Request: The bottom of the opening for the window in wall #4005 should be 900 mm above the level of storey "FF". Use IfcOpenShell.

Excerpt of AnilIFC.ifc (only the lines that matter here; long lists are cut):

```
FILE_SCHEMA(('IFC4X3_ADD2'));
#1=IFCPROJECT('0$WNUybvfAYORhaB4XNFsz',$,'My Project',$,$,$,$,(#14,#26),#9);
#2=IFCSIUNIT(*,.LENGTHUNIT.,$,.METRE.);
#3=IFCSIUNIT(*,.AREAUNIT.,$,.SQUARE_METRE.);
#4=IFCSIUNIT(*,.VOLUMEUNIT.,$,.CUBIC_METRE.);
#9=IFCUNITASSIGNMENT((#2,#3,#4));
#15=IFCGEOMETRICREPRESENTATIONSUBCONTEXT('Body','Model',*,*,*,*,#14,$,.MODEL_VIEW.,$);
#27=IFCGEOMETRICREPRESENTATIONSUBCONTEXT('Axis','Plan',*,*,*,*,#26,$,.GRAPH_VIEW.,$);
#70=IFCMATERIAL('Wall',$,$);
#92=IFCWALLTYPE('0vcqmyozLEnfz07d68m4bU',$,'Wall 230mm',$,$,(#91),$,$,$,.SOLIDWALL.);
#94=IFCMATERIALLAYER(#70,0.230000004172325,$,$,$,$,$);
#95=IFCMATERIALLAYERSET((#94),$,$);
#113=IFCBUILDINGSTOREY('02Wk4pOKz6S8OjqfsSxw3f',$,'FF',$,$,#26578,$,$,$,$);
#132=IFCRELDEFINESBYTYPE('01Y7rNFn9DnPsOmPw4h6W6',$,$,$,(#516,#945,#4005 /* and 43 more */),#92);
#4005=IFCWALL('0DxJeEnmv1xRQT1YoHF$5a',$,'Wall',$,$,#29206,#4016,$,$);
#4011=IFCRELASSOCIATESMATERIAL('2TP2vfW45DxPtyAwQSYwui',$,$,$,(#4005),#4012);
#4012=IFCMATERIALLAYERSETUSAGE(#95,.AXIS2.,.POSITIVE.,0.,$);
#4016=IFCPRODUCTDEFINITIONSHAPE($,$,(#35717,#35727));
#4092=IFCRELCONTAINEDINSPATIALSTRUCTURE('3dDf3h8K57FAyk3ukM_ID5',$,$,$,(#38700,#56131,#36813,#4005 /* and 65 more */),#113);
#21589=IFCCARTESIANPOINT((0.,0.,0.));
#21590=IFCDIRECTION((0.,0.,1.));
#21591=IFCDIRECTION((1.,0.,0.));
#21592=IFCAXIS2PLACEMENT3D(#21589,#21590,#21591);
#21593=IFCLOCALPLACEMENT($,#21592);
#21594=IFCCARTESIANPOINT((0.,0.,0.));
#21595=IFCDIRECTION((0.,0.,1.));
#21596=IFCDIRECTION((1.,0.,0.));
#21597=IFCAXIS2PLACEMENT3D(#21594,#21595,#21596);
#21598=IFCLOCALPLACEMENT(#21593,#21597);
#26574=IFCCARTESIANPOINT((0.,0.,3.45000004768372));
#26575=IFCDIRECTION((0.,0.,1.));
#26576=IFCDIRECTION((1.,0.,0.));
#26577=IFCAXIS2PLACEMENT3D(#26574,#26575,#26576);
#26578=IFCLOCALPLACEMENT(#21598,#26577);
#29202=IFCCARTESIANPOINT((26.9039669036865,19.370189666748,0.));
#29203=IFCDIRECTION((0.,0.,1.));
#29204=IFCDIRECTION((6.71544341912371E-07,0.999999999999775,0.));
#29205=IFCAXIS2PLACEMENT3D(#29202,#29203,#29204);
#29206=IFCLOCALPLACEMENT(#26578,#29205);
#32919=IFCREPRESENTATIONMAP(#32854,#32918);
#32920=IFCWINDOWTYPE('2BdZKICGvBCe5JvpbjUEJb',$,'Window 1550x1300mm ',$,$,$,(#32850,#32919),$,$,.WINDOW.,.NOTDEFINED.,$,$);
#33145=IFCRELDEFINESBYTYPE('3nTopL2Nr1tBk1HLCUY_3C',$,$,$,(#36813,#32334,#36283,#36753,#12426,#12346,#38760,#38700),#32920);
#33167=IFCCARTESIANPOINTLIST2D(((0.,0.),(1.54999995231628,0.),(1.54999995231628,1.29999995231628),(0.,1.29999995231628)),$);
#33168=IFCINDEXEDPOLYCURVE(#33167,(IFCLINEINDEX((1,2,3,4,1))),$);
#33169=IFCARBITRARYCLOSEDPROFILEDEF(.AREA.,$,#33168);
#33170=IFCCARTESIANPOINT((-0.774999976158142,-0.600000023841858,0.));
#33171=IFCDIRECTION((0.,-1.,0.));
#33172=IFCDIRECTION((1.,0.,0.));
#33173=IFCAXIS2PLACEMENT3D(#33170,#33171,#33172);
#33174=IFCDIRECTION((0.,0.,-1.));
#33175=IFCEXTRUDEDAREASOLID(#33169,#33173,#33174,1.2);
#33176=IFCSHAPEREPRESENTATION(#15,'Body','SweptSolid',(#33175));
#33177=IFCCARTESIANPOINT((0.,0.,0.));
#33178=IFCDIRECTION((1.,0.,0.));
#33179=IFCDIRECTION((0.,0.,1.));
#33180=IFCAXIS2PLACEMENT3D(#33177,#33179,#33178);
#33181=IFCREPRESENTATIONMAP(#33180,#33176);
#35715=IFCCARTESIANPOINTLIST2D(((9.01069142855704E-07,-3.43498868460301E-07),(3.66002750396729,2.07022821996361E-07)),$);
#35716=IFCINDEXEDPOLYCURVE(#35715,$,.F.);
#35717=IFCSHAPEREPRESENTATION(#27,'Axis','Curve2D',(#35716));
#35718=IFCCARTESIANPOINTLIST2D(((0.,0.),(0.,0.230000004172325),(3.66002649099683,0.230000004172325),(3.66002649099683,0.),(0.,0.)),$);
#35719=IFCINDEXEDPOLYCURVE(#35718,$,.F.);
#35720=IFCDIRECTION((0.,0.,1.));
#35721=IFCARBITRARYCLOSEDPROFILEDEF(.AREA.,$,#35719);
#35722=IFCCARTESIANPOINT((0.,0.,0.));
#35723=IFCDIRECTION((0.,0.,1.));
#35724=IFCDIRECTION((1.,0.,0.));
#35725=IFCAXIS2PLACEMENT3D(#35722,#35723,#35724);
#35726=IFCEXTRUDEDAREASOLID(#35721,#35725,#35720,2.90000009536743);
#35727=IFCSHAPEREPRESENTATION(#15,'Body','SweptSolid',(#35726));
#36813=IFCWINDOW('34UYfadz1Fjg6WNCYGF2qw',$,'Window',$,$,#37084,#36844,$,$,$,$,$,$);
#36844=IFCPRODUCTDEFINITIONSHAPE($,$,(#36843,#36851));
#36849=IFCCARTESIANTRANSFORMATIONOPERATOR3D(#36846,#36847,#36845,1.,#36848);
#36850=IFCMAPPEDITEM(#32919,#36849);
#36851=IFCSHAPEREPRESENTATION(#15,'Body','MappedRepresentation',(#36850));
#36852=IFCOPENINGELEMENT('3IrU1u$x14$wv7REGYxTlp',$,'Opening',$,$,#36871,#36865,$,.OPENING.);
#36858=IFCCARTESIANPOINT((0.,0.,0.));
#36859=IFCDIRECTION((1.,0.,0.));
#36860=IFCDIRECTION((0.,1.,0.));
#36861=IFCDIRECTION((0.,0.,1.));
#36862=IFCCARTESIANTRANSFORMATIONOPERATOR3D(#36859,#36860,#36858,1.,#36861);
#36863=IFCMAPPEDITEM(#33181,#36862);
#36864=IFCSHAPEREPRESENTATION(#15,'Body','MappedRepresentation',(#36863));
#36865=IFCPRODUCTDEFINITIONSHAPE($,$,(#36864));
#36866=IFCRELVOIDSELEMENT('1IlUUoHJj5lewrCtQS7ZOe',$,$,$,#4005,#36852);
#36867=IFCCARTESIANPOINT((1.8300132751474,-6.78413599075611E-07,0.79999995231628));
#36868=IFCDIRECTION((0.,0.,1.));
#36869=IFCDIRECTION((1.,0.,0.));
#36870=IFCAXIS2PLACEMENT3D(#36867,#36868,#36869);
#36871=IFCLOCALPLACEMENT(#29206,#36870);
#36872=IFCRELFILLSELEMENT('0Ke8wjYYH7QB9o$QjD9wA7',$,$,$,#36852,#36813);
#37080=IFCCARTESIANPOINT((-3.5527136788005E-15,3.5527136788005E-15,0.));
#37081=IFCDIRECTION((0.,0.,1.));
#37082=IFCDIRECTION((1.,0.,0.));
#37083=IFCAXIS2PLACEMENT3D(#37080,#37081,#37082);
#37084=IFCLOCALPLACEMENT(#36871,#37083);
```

```python
import numpy as np
import ifcopenshell
import ifcopenshell.api.geometry
import ifcopenshell.geom
import ifcopenshell.util.element
import ifcopenshell.util.placement
import ifcopenshell.util.shape
import ifcopenshell.util.unit

model = ifcopenshell.open("AnilIFC.ifc")
unit_scale = ifcopenshell.util.unit.calculate_unit_scale(model)

window = model.by_guid("34UYfadz1Fjg6WNCYGF2qw")
opening = window.FillsVoids[0].RelatingOpeningElement
storey = ifcopenshell.util.element.get_container(window, ifc_class="IfcBuildingStorey")
level = ifcopenshell.util.placement.get_local_placement(storey.ObjectPlacement)[2, 3]

# The opening's origin need not be at the sill, so measure its lowest point.
shape = ifcopenshell.geom.create_shape(ifcopenshell.geom.settings(), opening)
bottom = ifcopenshell.util.shape.get_shape_bottom_elevation(shape, shape.geometry) / unit_scale
dz = level + 0.9 - bottom

shift = np.array([0.0, 0.0, dz])
# The window is placed relative to its opening, so it follows when the opening moves.
matrix = ifcopenshell.util.placement.get_local_placement(opening.ObjectPlacement)
matrix[:3, 3] += shift
ifcopenshell.api.geometry.edit_object_placement(
    model, product=opening, matrix=matrix, is_si=False, should_transform_children=True
)

print(f"moved by {dz * unit_scale:+.3f} m")

model.write("AnilIFC-out.ifc")
```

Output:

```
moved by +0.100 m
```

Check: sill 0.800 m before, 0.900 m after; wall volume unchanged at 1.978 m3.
